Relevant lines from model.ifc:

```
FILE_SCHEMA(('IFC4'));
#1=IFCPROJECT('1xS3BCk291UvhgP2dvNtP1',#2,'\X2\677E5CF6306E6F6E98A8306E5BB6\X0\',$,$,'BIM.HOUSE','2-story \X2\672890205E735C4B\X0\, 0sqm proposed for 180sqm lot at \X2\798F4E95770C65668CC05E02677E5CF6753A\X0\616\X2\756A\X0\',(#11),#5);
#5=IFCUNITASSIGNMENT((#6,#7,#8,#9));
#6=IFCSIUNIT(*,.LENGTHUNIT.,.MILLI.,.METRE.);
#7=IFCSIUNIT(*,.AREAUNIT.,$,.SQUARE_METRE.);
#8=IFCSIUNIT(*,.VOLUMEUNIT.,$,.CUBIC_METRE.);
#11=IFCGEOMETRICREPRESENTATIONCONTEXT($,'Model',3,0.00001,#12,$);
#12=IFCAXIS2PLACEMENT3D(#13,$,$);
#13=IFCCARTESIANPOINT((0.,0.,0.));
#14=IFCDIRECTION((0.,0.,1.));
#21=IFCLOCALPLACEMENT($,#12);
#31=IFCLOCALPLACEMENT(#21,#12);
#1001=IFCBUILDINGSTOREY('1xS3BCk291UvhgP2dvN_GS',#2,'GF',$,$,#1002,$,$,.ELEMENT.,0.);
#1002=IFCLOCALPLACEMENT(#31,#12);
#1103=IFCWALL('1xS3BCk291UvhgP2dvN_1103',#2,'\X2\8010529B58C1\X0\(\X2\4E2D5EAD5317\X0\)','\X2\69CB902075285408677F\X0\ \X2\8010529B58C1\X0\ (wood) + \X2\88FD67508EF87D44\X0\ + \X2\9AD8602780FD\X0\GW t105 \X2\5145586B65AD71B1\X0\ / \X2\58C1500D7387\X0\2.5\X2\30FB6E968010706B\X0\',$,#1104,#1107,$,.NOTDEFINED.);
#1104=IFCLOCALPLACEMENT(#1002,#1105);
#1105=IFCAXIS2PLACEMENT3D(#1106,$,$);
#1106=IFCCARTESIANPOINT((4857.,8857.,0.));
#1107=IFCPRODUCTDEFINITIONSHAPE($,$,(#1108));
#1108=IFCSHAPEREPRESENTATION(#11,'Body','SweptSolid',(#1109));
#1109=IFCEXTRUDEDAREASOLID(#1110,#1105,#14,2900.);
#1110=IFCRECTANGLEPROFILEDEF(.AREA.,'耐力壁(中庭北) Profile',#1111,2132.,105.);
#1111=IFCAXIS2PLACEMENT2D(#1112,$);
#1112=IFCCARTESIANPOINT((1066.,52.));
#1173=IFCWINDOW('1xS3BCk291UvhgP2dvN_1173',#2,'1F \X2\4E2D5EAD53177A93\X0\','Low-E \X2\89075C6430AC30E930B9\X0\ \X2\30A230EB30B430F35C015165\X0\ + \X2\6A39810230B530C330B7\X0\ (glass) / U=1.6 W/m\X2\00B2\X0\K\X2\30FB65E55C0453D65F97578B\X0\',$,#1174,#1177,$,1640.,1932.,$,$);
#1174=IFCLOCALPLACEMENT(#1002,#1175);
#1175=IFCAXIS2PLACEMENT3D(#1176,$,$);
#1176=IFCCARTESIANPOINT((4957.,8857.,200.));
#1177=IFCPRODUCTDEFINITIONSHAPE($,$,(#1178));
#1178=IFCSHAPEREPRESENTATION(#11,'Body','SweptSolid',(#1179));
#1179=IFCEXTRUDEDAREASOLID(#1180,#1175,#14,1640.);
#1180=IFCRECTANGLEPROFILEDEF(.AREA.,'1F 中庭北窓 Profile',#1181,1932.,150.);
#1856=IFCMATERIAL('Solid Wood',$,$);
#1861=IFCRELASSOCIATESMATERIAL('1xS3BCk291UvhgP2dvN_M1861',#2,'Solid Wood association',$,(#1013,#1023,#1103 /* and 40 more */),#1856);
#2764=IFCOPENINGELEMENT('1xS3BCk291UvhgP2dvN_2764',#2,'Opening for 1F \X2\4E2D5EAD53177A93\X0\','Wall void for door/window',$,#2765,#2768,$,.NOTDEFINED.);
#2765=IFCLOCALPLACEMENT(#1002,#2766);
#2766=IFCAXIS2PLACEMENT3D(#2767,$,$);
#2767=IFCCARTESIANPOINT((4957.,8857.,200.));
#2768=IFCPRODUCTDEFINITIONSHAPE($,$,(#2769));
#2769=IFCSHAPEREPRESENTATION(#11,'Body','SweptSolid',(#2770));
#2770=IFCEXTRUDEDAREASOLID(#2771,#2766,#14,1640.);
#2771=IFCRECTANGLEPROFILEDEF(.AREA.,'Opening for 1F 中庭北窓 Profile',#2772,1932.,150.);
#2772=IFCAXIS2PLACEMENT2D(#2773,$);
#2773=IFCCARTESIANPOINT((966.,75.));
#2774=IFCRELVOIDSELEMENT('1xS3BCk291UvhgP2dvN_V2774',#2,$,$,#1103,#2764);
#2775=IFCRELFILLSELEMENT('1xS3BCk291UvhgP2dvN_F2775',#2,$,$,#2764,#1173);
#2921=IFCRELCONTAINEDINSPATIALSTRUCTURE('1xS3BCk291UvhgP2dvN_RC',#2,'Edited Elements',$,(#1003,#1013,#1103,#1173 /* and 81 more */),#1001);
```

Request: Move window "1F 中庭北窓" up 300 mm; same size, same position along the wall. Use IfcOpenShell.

```python
import numpy as np
import ifcopenshell
import ifcopenshell.api.geometry
import ifcopenshell.util.placement
import ifcopenshell.util.unit

model = ifcopenshell.open("model.ifc")
unit_scale = ifcopenshell.util.unit.calculate_unit_scale(model)

window = model.by_id(1173)
opening = window.FillsVoids[0].RelatingOpeningElement
dz = 0.3 / unit_scale

shift = np.array([0.0, 0.0, dz])
# The window is not placed relative to its opening, so move both.
for product in (opening, window):
    matrix = ifcopenshell.util.placement.get_local_placement(product.ObjectPlacement)
    matrix[:3, 3] += shift
    ifcopenshell.api.geometry.edit_object_placement(model, product=product, matrix=matrix, is_si=False)

print(f"moved by {dz * unit_scale:+.3f} m")

model.write("model_edited.ifc")
```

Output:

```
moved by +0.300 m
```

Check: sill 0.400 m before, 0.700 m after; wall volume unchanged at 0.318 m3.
